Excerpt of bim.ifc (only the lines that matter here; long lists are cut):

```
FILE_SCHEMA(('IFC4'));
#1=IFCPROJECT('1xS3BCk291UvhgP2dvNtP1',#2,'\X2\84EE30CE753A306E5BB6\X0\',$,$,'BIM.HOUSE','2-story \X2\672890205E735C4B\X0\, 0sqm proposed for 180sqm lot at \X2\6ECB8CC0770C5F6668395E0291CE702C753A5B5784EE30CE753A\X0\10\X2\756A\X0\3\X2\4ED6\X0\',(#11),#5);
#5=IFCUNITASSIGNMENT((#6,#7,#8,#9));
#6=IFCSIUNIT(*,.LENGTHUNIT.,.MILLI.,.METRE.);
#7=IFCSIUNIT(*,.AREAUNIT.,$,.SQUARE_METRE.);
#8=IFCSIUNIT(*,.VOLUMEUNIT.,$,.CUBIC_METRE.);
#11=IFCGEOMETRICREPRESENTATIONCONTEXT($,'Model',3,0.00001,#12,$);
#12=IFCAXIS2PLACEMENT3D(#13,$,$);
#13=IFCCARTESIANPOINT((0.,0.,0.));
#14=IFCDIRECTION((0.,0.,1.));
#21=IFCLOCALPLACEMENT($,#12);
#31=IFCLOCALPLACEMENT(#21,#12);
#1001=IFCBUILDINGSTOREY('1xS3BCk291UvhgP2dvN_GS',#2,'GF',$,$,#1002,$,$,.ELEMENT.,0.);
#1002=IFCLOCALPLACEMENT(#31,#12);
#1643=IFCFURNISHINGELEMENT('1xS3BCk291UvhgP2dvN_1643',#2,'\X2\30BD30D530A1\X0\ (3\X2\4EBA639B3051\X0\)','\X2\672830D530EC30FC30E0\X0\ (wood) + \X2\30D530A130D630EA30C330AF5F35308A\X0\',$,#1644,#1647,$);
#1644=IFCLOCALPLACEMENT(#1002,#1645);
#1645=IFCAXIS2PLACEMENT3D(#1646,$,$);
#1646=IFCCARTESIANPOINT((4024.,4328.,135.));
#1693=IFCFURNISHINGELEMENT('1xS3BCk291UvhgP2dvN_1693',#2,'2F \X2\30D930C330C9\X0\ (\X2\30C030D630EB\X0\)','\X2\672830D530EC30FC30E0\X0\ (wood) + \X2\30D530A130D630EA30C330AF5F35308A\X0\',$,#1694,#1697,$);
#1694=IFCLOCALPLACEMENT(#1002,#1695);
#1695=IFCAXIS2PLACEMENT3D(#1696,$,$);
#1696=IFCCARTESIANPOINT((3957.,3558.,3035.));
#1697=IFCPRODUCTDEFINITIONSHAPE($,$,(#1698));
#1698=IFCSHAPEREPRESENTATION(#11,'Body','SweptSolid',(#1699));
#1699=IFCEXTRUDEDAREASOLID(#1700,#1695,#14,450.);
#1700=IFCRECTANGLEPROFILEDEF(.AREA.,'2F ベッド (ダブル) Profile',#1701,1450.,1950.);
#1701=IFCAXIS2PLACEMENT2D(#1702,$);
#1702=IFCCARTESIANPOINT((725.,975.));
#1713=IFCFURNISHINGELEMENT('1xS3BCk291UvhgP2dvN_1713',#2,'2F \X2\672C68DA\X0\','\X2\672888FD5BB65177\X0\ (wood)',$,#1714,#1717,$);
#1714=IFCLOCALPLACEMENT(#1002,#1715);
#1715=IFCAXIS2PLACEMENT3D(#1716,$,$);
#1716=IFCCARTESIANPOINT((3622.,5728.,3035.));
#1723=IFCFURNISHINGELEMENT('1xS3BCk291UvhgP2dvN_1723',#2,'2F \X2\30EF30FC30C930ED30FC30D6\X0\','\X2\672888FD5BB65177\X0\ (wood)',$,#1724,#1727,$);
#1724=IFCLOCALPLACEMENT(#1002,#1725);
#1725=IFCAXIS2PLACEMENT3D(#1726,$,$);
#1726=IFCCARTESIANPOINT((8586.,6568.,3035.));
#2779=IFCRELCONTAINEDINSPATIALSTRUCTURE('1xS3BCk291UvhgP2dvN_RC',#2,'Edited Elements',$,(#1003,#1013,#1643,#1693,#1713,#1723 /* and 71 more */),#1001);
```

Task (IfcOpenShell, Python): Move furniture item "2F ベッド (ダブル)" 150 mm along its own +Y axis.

```python
import ifcopenshell
import ifcopenshell.api.geometry
import ifcopenshell.util.placement

model = ifcopenshell.open("bim.ifc")

item = model.by_guid("1xS3BCk291UvhgP2dvN_1693")
matrix = ifcopenshell.util.placement.get_local_placement(item.ObjectPlacement)
matrix[:3, 3] += matrix[:3, 1] * 150.0
ifcopenshell.api.geometry.edit_object_placement(model, product=item, matrix=matrix, is_si=False)

print(ifcopenshell.util.placement.get_local_placement(item.ObjectPlacement).round(3) + 0.0)

model.write("bim-out.ifc")
```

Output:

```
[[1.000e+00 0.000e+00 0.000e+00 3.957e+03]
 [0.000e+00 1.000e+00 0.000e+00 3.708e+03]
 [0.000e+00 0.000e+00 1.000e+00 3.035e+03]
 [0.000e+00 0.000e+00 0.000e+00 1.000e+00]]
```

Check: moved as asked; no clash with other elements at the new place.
